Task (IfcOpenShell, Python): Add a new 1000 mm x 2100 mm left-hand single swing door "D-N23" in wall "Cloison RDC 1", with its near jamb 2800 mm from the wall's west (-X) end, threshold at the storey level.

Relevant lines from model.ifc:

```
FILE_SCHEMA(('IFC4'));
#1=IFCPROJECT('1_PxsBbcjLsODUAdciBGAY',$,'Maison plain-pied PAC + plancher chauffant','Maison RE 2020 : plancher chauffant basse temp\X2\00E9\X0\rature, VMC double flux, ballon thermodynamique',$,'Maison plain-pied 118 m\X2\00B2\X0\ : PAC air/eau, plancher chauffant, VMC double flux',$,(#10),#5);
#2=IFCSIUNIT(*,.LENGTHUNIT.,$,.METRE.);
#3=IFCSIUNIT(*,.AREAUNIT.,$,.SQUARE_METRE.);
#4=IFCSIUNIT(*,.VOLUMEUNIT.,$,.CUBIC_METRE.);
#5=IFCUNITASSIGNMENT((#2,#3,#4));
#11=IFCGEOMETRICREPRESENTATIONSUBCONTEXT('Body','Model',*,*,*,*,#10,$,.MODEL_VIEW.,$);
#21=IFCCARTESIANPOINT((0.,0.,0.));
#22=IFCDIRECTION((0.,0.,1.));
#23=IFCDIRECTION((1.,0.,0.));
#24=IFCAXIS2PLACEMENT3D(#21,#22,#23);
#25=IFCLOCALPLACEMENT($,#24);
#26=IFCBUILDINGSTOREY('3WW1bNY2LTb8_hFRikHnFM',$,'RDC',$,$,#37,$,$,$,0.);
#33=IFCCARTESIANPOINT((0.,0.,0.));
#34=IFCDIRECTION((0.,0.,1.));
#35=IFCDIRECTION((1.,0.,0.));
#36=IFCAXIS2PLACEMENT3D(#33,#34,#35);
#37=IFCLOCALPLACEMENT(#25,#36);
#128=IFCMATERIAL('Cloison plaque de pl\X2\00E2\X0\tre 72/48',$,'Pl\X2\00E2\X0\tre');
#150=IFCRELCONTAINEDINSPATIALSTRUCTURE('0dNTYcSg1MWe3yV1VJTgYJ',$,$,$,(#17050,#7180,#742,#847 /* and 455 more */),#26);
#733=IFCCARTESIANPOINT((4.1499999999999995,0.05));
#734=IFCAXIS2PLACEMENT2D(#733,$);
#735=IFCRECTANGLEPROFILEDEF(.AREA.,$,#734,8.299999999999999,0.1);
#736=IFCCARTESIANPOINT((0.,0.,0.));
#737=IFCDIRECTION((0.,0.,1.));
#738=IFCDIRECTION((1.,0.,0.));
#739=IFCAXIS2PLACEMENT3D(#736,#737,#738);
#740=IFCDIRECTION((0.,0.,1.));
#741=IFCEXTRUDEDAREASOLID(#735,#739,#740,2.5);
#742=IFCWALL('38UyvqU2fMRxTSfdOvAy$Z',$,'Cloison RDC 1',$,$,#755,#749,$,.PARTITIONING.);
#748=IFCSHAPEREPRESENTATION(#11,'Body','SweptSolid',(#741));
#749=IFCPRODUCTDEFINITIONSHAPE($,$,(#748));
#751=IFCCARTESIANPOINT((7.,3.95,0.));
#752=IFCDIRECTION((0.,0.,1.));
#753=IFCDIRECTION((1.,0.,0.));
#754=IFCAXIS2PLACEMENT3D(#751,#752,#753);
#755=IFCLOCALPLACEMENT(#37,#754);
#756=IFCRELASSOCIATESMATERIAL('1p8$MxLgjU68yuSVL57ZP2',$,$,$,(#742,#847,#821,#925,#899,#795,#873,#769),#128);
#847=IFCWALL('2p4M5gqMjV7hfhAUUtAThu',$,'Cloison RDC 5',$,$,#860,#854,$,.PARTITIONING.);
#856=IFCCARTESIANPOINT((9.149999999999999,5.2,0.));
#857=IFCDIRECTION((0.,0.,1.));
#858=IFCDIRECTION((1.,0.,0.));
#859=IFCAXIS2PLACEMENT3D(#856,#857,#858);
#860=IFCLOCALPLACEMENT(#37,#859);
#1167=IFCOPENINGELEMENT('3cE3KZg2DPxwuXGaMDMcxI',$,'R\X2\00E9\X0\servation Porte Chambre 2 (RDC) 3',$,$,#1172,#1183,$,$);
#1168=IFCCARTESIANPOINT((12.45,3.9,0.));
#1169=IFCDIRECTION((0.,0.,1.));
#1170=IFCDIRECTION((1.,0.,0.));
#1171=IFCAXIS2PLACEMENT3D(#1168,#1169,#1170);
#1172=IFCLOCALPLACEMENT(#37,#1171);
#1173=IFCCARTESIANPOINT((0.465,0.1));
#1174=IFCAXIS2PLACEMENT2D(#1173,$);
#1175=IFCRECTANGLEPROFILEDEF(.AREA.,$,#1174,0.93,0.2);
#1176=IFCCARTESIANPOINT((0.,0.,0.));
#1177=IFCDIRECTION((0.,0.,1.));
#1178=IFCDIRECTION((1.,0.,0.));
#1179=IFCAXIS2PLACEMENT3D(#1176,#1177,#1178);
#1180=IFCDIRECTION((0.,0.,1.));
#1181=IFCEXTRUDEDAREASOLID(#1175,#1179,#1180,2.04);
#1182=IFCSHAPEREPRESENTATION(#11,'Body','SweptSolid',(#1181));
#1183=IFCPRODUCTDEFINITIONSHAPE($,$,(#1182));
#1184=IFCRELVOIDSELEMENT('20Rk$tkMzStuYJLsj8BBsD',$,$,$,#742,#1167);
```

```python
import numpy as np
import ifcopenshell
import ifcopenshell.api.feature
import ifcopenshell.api.geometry
import ifcopenshell.api.root
import ifcopenshell.api.spatial
import ifcopenshell.geom
import ifcopenshell.util.element
import ifcopenshell.util.placement
import ifcopenshell.util.representation
import ifcopenshell.util.shape
import ifcopenshell.util.unit

model = ifcopenshell.open("model.ifc")
unit_scale = ifcopenshell.util.unit.calculate_unit_scale(model)
settings = ifcopenshell.geom.settings()


def volume(element):
    """Net volume in cubic metres, openings subtracted."""
    shape = ifcopenshell.geom.create_shape(settings, element)
    return ifcopenshell.util.shape.get_volume(shape.geometry)


wall = model.by_guid("38UyvqU2fMRxTSfdOvAy$Z")
storey = ifcopenshell.util.element.get_container(wall, ifc_class="IfcBuildingStorey")
context = ifcopenshell.util.representation.get_context(model, "Model", "Body", "MODEL_VIEW")
before = volume(wall)

width, height, from_end, sill = 1, 2.1, 2.8, 0.0  # metres

# The wall runs along its own X axis, and the end named is its -X end.
wall_shape = ifcopenshell.geom.create_shape(settings, wall)
x, y, z = ifcopenshell.util.shape.get_vertices(wall_shape.geometry).T
start = x.min() + from_end
face, thickness = float(y.min()), float(y.max() - y.min())
wall_matrix = ifcopenshell.util.placement.get_local_placement(wall.ObjectPlacement)
level = ifcopenshell.util.placement.get_local_placement(storey.ObjectPlacement)[2, 3]


def in_wall(x, y):
    """Placement at x, y metres in the wall's axes, at sill height."""
    matrix = wall_matrix.copy()
    matrix[:, 3] = wall_matrix @ np.array([x / unit_scale, y / unit_scale, 0.0, 1.0])
    matrix[2, 3] = level + sill / unit_scale
    return matrix


# Opening: a box that overshoots both wall faces by 50 mm.
opening = ifcopenshell.api.root.create_entity(model, ifc_class="IfcOpeningElement", predefined_type="OPENING")
box = ifcopenshell.api.geometry.add_wall_representation(
    model, context=context, length=width, height=height, thickness=thickness + 0.1
)
ifcopenshell.api.geometry.assign_representation(model, product=opening, representation=box)
ifcopenshell.api.geometry.edit_object_placement(model, product=opening, matrix=in_wall(start, face - 0.05), is_si=False)
ifcopenshell.api.feature.add_feature(model, feature=opening, element=wall)

door = ifcopenshell.api.root.create_entity(model, ifc_class="IfcDoor", name="D-N23", predefined_type="DOOR")
door.OverallWidth, door.OverallHeight = width / unit_scale, height / unit_scale
door.OperationType = "SINGLE_SWING_LEFT"
body = ifcopenshell.api.geometry.add_door_representation(
    model,
    context=context,
    overall_width=door.OverallWidth,
    overall_height=door.OverallHeight,
    operation_type="SINGLE_SWING_LEFT",
    lining_properties={"LiningDepth": thickness / unit_scale, "ThresholdDepth": thickness / unit_scale},
)
ifcopenshell.api.geometry.assign_representation(model, product=door, representation=body)
ifcopenshell.api.spatial.assign_container(model, products=[door], relating_structure=storey)
ifcopenshell.api.feature.add_filling(model, opening=opening, element=door)

# The lining spans the wall, so the door starts at the wall face.
ifcopenshell.api.geometry.edit_object_placement(model, product=door, matrix=in_wall(start, face), is_si=False)

after = volume(wall)

print(f"wall volume {before:.3f} -> {after:.3f} m3")

model.write("model_edited.ifc")
```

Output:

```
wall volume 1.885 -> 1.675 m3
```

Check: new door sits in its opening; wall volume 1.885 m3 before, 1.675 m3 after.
